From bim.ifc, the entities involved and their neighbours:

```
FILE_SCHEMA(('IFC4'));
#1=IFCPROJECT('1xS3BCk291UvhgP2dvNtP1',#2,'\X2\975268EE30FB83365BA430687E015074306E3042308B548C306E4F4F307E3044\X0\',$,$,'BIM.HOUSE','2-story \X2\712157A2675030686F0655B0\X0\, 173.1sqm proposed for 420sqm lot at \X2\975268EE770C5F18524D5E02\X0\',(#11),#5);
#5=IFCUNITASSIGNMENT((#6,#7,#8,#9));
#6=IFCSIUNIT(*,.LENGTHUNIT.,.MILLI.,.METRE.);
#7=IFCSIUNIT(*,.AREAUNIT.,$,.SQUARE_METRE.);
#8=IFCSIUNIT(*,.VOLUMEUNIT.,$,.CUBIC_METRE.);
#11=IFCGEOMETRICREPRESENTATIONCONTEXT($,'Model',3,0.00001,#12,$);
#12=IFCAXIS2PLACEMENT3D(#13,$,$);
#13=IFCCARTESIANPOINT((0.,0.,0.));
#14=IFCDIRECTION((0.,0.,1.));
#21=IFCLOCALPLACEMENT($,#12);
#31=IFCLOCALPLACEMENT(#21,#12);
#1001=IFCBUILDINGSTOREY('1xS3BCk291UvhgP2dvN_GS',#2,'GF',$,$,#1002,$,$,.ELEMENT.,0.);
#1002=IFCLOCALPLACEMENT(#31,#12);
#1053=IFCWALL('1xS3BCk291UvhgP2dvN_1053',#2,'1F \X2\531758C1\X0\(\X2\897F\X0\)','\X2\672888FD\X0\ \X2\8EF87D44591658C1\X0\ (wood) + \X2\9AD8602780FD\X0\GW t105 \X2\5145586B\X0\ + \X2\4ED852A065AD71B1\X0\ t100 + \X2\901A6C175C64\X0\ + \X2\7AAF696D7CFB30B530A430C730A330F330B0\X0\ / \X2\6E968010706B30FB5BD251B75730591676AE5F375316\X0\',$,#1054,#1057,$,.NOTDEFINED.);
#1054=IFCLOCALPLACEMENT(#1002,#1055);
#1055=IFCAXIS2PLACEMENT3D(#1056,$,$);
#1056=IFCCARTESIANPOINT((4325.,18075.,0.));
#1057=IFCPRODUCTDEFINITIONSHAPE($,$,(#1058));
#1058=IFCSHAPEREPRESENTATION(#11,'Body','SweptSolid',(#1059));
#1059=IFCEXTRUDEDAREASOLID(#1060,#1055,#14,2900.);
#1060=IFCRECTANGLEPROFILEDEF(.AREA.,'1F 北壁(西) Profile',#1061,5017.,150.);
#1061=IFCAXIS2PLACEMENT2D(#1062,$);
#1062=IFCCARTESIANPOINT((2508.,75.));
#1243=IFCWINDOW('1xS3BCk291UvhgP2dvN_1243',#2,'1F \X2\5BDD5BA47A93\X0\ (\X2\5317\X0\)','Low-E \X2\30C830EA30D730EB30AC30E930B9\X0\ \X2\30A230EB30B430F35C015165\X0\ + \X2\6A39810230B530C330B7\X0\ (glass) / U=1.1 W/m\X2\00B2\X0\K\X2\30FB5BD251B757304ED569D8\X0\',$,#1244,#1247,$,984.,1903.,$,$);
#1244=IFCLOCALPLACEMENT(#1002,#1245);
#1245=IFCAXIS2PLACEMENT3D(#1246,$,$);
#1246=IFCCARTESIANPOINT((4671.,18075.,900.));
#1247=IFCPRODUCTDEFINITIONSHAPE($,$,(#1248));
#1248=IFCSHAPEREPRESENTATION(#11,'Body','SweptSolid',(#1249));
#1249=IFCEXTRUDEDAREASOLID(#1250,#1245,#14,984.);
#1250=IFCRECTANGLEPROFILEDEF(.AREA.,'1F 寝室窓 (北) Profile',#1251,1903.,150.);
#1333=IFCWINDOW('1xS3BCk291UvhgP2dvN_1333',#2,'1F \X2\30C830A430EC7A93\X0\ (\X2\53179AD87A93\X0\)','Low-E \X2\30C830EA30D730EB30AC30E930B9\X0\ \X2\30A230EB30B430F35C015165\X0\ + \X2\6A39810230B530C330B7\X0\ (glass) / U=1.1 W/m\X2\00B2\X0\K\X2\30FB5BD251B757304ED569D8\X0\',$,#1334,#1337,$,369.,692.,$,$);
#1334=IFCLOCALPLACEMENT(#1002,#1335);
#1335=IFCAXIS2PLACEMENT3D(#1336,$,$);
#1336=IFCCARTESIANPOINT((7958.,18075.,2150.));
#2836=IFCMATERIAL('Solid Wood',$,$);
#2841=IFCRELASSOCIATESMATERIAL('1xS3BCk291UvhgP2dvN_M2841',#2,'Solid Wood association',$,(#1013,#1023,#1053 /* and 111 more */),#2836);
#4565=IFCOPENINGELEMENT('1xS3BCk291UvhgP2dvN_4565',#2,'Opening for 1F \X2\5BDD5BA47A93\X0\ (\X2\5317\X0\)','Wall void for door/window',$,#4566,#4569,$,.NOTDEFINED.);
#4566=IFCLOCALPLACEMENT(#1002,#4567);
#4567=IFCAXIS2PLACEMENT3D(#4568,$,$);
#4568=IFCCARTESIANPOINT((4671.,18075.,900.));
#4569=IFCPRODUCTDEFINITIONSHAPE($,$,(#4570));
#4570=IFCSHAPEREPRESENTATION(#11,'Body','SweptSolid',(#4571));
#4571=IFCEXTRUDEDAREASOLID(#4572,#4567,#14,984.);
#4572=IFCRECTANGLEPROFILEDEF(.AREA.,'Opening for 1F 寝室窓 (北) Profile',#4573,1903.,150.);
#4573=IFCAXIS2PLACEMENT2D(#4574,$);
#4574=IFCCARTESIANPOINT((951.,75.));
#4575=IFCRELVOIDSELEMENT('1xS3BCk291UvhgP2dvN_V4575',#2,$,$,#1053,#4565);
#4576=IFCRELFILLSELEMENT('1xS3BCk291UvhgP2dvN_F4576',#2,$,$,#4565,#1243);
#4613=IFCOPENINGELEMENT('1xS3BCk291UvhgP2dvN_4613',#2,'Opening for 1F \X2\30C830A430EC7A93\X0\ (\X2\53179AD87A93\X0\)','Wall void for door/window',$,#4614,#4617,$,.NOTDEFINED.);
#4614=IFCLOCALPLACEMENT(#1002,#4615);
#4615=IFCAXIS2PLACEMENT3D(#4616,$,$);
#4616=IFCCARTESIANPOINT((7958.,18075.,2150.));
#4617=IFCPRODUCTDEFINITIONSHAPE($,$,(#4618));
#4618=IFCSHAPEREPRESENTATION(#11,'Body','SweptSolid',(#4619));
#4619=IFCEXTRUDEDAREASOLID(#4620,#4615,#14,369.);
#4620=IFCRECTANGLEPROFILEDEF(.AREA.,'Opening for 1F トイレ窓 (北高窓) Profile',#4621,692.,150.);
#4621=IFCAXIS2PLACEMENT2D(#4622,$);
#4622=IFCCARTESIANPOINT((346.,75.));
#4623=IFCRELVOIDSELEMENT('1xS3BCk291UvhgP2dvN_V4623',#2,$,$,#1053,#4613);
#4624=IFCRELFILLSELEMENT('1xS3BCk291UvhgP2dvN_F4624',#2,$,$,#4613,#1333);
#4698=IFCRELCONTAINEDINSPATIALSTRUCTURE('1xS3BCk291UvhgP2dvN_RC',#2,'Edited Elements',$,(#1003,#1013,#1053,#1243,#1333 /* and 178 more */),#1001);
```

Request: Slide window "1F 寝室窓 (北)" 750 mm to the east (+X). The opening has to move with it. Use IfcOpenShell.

```python
import ifcopenshell
import ifcopenshell.api.geometry
import ifcopenshell.util.placement

model = ifcopenshell.open("bim.ifc")

window = model.by_guid("1xS3BCk291UvhgP2dvN_1243")
opening = window.FillsVoids[0].RelatingOpeningElement
wall = opening.VoidsElements[0].RelatingBuildingElement

wall_matrix = ifcopenshell.util.placement.get_local_placement(wall.ObjectPlacement)
shift = wall_matrix[:3, 0] * 750.0
before = ifcopenshell.util.placement.get_local_placement(window.ObjectPlacement)[:3, 3].copy()

# The window is not placed relative to its opening, so move both.
for product in (opening, window):
    matrix = ifcopenshell.util.placement.get_local_placement(product.ObjectPlacement)
    matrix[:3, 3] += shift
    ifcopenshell.api.geometry.edit_object_placement(model, product=product, matrix=matrix, is_si=False)

after = ifcopenshell.util.placement.get_local_placement(window.ObjectPlacement)[:3, 3]
print("window moved by", (after - before).round(3) + 0.0)

model.write("bim_rev.ifc")
```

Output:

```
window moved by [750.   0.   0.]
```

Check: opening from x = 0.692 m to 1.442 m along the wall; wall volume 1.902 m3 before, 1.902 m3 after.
